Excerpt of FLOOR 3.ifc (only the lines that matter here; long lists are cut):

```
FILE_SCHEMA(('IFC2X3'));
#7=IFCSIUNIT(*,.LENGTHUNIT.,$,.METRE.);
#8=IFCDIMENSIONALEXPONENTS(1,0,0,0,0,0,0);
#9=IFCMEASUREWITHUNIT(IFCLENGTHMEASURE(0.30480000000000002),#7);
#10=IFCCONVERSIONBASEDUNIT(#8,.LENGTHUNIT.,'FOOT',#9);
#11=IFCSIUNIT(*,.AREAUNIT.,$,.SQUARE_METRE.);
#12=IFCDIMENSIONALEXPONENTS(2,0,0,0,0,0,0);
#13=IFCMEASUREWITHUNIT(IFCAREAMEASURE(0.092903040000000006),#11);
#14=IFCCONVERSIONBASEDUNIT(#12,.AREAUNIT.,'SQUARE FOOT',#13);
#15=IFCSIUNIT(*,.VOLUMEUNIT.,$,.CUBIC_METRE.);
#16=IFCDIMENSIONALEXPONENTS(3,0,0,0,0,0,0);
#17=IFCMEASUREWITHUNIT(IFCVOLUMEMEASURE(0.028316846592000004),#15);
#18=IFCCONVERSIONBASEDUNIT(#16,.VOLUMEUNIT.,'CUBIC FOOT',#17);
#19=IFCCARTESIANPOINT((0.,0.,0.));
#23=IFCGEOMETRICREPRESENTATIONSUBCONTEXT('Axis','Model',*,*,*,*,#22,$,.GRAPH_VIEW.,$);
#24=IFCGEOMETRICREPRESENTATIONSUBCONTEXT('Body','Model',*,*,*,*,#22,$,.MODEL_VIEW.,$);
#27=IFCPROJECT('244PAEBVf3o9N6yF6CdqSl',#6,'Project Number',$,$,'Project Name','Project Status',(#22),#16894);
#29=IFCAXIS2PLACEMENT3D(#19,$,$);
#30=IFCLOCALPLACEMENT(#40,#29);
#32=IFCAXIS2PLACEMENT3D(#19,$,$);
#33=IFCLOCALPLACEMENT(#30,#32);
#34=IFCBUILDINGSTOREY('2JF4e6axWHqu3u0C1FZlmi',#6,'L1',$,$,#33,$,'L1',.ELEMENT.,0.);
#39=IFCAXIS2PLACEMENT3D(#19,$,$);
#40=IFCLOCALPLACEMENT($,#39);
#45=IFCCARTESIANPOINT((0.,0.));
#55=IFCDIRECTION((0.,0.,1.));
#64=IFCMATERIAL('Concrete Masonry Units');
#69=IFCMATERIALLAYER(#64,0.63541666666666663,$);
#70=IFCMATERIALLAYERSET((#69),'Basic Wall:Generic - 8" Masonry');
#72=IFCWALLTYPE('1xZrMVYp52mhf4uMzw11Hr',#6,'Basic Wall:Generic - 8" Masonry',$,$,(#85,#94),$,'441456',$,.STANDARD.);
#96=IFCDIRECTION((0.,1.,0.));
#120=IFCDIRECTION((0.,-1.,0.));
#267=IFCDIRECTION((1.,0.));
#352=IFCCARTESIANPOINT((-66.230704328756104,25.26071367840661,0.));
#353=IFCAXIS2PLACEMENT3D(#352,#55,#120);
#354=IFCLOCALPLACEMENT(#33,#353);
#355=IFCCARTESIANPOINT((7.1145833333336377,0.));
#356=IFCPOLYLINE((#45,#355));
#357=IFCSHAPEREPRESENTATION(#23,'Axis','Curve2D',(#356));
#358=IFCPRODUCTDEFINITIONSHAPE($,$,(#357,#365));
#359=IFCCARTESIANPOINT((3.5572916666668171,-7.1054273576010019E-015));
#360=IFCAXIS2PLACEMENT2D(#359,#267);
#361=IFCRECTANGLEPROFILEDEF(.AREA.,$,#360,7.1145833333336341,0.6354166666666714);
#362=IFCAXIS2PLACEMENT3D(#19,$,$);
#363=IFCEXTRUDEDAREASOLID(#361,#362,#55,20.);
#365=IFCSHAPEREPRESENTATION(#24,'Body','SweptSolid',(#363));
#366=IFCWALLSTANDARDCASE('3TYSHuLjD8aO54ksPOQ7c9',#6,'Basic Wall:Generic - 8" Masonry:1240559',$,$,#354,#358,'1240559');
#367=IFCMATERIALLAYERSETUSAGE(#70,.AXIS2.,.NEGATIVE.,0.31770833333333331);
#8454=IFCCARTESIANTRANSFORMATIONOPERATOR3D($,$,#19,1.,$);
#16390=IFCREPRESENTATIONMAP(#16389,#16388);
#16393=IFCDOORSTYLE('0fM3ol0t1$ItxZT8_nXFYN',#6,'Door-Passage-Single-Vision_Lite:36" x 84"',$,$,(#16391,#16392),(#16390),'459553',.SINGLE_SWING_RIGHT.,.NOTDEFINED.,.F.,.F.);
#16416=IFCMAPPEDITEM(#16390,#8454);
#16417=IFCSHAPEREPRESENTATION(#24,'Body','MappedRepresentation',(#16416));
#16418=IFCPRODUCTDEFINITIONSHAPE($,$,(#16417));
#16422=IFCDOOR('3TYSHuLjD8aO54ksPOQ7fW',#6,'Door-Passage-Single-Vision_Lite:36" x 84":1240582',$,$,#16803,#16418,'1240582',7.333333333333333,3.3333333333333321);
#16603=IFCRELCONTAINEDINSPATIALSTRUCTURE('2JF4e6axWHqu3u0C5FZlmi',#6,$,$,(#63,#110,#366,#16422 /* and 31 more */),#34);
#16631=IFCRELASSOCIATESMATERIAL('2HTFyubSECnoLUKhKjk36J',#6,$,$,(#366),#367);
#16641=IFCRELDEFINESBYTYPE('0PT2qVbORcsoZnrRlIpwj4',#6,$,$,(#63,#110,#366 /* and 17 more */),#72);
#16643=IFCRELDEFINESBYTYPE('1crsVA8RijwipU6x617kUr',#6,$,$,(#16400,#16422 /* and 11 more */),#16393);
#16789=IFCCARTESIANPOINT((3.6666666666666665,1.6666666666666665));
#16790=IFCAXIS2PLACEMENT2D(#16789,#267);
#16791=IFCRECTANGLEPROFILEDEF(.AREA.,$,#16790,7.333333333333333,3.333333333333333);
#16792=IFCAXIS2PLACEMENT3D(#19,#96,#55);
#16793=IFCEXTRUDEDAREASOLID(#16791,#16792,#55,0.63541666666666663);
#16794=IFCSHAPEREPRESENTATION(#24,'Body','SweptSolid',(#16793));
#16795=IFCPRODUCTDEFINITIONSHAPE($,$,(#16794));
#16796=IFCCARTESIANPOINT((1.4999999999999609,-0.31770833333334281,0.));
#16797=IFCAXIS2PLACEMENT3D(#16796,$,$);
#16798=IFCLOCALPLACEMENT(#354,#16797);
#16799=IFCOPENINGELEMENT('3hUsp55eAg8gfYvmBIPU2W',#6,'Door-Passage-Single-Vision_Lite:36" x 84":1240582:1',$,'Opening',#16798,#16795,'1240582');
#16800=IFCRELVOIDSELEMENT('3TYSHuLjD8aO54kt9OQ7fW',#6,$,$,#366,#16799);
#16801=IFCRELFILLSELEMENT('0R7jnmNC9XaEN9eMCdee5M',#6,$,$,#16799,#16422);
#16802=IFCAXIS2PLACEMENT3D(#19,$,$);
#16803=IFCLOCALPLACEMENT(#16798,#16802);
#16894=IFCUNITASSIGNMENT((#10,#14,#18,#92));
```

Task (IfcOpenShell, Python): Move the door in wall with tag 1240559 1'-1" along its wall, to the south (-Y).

```python
import ifcopenshell
import ifcopenshell.api.geometry
import ifcopenshell.util.placement
import ifcopenshell.util.unit

model = ifcopenshell.open("FLOOR 3.ifc")
unit_scale = ifcopenshell.util.unit.calculate_unit_scale(model)

door = model.by_guid("3TYSHuLjD8aO54ksPOQ7fW")
opening = door.FillsVoids[0].RelatingOpeningElement
wall = opening.VoidsElements[0].RelatingBuildingElement

wall_matrix = ifcopenshell.util.placement.get_local_placement(wall.ObjectPlacement)
shift = wall_matrix[:3, 0] * 13 * 0.0254 / unit_scale
before = ifcopenshell.util.placement.get_local_placement(door.ObjectPlacement)[:3, 3].copy()

# The door is placed relative to its opening, so it follows when the opening moves.
matrix = ifcopenshell.util.placement.get_local_placement(opening.ObjectPlacement)
matrix[:3, 3] += shift
ifcopenshell.api.geometry.edit_object_placement(
    model, product=opening, matrix=matrix, is_si=False, should_transform_children=True
)

after = ifcopenshell.util.placement.get_local_placement(door.ObjectPlacement)[:3, 3]
print("door moved by", (after - before).round(3) + 0.0)

model.write("FLOOR 3_updated.ifc")
```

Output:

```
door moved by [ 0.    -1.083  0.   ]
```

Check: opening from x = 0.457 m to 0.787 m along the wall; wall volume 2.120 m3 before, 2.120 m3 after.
